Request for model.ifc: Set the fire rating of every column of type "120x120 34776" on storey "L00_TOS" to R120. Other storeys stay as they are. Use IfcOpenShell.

First a look at what the model holds.

```python
import ifcopenshell
import ifcopenshell.util.element

model = ifcopenshell.open("model.ifc")
print(model.schema)
storey = next(s for s in model.by_type("IfcBuildingStorey") if s.Name == "L00_TOS")
columns = [e for e in ifcopenshell.util.element.get_decomposition(storey) if e.is_a("IfcColumn")]
seen = {}
for e in columns:
    element_type = ifcopenshell.util.element.get_type(e)
    key = (element_type.Name if element_type != e and element_type else None, ifcopenshell.util.element.get_pset(e, "Pset_ColumnCommon", "FireRating"))
    seen[key] = seen.get(key, 0) + 1
for (name, value), count in sorted(seen.items(), key=str):
    print(count, "x", name, "|", value)
```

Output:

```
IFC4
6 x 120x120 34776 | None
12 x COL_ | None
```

```python
import ifcopenshell
import ifcopenshell.api.pset
import ifcopenshell.util.element

model = ifcopenshell.open("model.ifc")

storey = next(s for s in model.by_type("IfcBuildingStorey") if s.Name == "L00_TOS")
columns = [e for e in ifcopenshell.util.element.get_decomposition(storey) if e.is_a("IfcColumn")]

count = 0
for e in columns:
    element_type = ifcopenshell.util.element.get_type(e)
    if element_type in (None, e) or element_type.Name != "120x120 34776":
        continue
    # add_pset returns the element's existing set when there is one.
    pset = ifcopenshell.api.pset.add_pset(model, product=e, name="Pset_ColumnCommon")
    ifcopenshell.api.pset.edit_pset(model, pset=pset, properties={"FireRating": "R120"})
    count += 1

print(count, "columns updated")

model.write("model_rev.ifc")
```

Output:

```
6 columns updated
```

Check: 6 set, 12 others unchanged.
